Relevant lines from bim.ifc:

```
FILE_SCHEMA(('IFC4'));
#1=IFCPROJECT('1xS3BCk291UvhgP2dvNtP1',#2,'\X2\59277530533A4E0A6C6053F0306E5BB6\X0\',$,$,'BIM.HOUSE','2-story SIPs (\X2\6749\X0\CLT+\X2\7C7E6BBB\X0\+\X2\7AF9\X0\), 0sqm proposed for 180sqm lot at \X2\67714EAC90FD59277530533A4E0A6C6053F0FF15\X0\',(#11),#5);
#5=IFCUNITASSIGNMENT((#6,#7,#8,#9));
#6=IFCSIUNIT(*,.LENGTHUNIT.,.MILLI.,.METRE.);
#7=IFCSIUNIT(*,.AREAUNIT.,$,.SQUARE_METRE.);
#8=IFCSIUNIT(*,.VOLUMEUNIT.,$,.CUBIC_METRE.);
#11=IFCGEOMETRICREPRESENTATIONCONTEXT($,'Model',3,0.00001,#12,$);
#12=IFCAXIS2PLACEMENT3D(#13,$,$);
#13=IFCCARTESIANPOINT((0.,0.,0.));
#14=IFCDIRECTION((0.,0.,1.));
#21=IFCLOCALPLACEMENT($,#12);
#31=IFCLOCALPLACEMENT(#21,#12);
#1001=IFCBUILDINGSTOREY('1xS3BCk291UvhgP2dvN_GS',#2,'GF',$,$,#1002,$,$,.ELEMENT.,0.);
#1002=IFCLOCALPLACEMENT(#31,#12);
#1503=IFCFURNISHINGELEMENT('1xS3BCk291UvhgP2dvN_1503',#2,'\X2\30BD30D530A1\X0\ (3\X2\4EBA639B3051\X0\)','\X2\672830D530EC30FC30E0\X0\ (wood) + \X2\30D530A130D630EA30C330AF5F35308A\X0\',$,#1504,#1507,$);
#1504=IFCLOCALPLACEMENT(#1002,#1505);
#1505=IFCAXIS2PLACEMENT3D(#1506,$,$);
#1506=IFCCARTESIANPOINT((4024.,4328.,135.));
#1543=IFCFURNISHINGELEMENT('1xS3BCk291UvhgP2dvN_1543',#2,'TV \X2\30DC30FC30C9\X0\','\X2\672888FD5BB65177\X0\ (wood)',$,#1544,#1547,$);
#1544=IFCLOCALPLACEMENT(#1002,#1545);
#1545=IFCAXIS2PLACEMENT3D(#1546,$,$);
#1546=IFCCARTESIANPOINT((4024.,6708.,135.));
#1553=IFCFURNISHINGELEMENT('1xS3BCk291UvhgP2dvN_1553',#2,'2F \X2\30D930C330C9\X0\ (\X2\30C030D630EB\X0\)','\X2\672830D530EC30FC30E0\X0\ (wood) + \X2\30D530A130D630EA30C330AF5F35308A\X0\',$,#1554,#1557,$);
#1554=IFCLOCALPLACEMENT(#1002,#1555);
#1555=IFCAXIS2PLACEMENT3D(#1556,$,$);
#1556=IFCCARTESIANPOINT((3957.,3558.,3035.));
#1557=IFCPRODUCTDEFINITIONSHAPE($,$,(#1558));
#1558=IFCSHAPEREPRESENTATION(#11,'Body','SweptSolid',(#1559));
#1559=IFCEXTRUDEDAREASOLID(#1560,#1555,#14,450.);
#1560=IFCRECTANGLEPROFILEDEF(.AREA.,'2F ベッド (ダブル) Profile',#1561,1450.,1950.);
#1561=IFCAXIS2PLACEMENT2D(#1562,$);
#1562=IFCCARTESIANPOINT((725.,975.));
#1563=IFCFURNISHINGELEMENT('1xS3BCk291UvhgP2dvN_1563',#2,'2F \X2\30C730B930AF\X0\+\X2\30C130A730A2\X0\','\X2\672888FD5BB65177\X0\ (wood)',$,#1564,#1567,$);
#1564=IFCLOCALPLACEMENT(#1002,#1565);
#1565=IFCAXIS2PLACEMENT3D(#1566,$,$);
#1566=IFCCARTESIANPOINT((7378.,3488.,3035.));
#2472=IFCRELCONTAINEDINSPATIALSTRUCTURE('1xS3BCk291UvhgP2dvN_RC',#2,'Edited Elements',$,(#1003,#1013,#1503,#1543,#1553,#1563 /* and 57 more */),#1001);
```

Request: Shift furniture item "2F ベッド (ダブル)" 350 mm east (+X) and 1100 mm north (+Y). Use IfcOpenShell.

```python
import ifcopenshell
import ifcopenshell.api.geometry
import ifcopenshell.util.placement

model = ifcopenshell.open("bim.ifc")

item = model.by_guid("1xS3BCk291UvhgP2dvN_1553")
matrix = ifcopenshell.util.placement.get_local_placement(item.ObjectPlacement)
matrix[0, 3] += 350.0
matrix[1, 3] += 1100.0
ifcopenshell.api.geometry.edit_object_placement(model, product=item, matrix=matrix, is_si=False)

print(ifcopenshell.util.placement.get_local_placement(item.ObjectPlacement).round(3) + 0.0)

model.write("bim_v2.ifc")
```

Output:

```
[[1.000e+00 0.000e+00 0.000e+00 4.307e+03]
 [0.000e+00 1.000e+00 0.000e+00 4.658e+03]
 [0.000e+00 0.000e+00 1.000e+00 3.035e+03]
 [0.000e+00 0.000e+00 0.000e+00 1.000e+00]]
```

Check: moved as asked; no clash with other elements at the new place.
